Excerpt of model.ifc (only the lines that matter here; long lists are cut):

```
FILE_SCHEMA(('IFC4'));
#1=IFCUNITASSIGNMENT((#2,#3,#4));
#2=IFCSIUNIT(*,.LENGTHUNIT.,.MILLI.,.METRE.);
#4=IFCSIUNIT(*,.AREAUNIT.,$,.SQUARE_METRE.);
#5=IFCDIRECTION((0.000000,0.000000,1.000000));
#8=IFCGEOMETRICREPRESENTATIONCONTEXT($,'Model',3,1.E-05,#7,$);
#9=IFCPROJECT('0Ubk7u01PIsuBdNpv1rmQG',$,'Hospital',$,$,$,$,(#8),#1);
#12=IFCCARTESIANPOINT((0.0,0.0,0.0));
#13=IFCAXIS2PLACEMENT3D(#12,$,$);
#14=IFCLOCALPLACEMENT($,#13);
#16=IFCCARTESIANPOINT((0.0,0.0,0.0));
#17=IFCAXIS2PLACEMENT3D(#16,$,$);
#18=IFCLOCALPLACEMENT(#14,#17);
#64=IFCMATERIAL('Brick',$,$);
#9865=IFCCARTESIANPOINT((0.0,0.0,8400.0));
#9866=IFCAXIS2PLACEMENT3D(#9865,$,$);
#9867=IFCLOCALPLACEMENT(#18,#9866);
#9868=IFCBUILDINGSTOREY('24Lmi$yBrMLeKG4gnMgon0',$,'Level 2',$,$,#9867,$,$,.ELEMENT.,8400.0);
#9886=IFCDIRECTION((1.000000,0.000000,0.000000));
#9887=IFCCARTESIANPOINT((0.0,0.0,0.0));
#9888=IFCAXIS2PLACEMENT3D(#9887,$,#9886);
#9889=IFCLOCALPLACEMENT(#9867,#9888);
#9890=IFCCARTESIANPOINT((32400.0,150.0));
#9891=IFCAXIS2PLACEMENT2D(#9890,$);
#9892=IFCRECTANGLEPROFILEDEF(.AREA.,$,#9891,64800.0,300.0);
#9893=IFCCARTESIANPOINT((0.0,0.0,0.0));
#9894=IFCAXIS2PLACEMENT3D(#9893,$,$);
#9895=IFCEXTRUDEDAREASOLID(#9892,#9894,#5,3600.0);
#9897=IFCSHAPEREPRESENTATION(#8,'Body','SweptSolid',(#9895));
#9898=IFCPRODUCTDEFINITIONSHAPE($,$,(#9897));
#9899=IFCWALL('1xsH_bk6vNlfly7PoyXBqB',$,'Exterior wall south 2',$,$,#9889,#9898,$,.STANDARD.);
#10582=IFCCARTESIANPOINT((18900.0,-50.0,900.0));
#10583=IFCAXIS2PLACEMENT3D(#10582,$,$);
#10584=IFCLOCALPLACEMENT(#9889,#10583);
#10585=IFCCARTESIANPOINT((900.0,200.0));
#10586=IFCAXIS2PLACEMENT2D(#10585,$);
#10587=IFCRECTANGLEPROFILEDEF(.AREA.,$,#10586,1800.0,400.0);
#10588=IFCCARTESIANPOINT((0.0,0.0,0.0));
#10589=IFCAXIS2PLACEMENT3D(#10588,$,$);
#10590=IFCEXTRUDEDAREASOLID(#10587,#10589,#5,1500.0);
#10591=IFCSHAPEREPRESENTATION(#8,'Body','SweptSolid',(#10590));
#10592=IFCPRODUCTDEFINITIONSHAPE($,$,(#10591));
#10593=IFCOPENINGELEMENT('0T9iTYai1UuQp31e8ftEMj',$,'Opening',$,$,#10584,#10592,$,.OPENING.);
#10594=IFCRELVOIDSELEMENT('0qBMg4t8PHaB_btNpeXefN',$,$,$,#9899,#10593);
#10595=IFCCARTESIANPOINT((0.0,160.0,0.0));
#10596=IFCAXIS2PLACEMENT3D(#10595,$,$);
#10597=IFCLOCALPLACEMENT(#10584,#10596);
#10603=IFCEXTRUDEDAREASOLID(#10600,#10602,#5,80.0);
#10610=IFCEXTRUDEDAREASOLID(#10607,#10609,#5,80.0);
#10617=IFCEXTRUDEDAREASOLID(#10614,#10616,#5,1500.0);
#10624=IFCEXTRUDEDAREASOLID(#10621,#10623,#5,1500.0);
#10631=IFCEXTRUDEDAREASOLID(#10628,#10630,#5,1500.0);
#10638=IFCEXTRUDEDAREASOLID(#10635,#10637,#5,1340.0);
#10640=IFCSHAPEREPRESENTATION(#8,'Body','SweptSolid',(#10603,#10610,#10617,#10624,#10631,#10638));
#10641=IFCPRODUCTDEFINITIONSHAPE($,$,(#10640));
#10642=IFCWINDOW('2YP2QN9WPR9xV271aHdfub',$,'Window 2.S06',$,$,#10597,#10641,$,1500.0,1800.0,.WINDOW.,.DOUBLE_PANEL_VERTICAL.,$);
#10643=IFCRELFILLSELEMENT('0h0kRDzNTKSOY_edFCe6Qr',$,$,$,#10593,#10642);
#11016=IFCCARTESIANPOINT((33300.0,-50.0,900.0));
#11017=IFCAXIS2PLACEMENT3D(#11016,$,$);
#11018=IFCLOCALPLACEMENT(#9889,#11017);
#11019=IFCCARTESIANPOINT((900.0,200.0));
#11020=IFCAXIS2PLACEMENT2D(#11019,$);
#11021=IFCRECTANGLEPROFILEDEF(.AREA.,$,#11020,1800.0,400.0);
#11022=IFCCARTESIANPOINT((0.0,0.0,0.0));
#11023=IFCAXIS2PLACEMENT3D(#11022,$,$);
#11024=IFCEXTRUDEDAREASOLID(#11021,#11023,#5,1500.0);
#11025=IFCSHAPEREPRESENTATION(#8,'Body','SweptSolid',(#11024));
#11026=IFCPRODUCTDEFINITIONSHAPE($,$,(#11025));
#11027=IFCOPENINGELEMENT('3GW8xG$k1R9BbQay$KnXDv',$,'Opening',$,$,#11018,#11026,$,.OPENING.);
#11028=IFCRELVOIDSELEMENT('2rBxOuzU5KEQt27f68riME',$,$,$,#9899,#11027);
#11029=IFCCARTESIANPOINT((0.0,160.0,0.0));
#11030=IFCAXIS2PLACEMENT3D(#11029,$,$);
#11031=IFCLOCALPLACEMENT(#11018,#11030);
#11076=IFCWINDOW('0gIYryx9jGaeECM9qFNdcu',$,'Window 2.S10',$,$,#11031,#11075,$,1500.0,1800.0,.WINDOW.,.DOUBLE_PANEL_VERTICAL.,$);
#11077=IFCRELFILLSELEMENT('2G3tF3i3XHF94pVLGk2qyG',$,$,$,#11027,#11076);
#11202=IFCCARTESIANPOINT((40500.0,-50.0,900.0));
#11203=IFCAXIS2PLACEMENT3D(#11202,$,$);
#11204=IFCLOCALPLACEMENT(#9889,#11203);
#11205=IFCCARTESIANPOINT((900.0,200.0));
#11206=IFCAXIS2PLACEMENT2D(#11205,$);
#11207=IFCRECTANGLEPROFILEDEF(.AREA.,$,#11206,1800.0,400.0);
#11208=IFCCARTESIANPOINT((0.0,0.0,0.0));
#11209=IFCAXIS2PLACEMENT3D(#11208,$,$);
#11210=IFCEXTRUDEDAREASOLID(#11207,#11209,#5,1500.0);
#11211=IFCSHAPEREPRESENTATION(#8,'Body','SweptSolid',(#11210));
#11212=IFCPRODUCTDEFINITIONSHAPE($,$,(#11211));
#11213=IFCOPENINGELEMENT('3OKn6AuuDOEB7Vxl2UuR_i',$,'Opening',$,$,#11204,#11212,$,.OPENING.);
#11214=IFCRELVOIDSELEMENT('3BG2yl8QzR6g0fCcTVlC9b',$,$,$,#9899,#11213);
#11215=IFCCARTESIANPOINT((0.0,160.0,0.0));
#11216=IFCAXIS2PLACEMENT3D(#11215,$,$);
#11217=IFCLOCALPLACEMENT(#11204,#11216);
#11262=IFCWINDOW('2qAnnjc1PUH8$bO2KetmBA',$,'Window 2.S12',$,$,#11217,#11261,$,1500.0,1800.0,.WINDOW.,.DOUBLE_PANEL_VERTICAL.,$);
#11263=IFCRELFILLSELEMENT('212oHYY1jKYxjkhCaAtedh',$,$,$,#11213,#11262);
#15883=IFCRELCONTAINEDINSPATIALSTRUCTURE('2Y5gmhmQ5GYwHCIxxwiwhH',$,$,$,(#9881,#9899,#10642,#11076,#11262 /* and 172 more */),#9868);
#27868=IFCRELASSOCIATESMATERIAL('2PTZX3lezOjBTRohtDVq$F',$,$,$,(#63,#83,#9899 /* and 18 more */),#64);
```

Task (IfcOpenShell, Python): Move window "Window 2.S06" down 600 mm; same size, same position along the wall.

```python
import numpy as np
import ifcopenshell
import ifcopenshell.api.geometry
import ifcopenshell.util.placement
import ifcopenshell.util.unit

model = ifcopenshell.open("model.ifc")
unit_scale = ifcopenshell.util.unit.calculate_unit_scale(model)

window = model.by_guid("2YP2QN9WPR9xV271aHdfub")
opening = window.FillsVoids[0].RelatingOpeningElement
dz = -0.6 / unit_scale

shift = np.array([0.0, 0.0, dz])
# The window is placed relative to its opening, so it follows when the opening moves.
matrix = ifcopenshell.util.placement.get_local_placement(opening.ObjectPlacement)
matrix[:3, 3] += shift
ifcopenshell.api.geometry.edit_object_placement(
    model, product=opening, matrix=matrix, is_si=False, should_transform_children=True
)

print(f"moved by {dz * unit_scale:+.3f} m")

model.write("model-out.ifc")
```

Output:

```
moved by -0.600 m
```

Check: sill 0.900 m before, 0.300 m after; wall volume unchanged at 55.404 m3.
